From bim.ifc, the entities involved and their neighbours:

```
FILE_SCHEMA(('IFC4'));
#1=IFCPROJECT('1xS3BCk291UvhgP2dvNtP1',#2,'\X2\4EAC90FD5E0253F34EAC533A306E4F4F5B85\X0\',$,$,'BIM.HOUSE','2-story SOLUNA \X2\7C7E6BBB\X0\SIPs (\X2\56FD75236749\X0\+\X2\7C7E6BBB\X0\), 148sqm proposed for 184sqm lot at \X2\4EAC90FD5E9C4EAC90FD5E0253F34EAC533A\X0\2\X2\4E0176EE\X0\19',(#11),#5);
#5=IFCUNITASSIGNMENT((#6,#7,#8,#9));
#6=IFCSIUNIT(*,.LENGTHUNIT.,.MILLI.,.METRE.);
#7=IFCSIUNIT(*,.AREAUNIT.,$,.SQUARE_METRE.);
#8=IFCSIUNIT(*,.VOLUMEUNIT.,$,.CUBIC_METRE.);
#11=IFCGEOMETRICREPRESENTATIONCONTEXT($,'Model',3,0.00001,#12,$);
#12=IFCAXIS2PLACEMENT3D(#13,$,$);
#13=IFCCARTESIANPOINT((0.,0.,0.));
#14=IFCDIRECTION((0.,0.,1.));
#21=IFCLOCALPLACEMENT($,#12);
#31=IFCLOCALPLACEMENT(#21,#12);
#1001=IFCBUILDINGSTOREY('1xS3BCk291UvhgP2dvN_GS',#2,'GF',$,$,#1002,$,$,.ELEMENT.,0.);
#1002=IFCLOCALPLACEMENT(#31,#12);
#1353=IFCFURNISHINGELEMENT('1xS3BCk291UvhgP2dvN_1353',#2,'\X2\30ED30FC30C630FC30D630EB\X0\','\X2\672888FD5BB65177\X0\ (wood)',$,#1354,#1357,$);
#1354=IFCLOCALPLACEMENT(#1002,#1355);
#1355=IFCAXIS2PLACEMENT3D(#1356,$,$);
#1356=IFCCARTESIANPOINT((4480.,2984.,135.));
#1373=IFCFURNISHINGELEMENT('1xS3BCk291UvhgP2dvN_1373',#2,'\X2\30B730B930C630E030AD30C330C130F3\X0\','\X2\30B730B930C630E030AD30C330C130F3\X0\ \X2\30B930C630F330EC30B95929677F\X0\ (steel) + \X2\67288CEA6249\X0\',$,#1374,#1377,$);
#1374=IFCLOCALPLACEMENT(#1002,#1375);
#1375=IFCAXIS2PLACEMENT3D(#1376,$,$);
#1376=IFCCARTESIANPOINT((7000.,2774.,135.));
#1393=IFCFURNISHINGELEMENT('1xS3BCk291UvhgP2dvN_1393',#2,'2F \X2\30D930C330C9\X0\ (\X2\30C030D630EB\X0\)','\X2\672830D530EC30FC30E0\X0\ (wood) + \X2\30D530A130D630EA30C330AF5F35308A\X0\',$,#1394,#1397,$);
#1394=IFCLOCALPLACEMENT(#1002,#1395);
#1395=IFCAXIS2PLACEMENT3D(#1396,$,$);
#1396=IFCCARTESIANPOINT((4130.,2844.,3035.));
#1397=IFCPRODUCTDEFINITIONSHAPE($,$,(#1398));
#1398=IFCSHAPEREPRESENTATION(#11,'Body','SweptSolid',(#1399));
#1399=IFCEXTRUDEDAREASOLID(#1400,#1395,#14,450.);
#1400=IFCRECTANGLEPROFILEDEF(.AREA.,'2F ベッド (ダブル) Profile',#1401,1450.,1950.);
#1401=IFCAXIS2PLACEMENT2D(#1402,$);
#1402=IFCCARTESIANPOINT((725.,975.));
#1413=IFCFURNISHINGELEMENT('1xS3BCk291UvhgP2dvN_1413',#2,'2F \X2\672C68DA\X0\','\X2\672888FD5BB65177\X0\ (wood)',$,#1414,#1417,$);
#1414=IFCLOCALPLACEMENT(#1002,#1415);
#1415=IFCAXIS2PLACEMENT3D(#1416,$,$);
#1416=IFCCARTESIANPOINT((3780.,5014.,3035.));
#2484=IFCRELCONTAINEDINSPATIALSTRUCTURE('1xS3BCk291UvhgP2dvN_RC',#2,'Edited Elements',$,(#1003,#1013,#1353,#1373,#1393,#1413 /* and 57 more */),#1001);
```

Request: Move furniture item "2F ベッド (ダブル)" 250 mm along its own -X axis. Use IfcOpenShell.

```python
import ifcopenshell
import ifcopenshell.api.geometry
import ifcopenshell.util.placement
import ifcopenshell.util.unit

model = ifcopenshell.open("bim.ifc")
unit_scale = ifcopenshell.util.unit.calculate_unit_scale(model)

item = model.by_id(1393)
matrix = ifcopenshell.util.placement.get_local_placement(item.ObjectPlacement)
matrix[:3, 3] -= matrix[:3, 0] * 0.25 / unit_scale
ifcopenshell.api.geometry.edit_object_placement(model, product=item, matrix=matrix, is_si=False)

print(ifcopenshell.util.placement.get_local_placement(item.ObjectPlacement).round(3) + 0.0)

model.write("bim_v2.ifc")
```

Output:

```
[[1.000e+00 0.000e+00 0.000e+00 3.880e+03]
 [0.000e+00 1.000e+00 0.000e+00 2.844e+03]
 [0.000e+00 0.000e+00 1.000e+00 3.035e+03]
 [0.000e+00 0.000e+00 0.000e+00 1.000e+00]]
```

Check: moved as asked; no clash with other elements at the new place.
